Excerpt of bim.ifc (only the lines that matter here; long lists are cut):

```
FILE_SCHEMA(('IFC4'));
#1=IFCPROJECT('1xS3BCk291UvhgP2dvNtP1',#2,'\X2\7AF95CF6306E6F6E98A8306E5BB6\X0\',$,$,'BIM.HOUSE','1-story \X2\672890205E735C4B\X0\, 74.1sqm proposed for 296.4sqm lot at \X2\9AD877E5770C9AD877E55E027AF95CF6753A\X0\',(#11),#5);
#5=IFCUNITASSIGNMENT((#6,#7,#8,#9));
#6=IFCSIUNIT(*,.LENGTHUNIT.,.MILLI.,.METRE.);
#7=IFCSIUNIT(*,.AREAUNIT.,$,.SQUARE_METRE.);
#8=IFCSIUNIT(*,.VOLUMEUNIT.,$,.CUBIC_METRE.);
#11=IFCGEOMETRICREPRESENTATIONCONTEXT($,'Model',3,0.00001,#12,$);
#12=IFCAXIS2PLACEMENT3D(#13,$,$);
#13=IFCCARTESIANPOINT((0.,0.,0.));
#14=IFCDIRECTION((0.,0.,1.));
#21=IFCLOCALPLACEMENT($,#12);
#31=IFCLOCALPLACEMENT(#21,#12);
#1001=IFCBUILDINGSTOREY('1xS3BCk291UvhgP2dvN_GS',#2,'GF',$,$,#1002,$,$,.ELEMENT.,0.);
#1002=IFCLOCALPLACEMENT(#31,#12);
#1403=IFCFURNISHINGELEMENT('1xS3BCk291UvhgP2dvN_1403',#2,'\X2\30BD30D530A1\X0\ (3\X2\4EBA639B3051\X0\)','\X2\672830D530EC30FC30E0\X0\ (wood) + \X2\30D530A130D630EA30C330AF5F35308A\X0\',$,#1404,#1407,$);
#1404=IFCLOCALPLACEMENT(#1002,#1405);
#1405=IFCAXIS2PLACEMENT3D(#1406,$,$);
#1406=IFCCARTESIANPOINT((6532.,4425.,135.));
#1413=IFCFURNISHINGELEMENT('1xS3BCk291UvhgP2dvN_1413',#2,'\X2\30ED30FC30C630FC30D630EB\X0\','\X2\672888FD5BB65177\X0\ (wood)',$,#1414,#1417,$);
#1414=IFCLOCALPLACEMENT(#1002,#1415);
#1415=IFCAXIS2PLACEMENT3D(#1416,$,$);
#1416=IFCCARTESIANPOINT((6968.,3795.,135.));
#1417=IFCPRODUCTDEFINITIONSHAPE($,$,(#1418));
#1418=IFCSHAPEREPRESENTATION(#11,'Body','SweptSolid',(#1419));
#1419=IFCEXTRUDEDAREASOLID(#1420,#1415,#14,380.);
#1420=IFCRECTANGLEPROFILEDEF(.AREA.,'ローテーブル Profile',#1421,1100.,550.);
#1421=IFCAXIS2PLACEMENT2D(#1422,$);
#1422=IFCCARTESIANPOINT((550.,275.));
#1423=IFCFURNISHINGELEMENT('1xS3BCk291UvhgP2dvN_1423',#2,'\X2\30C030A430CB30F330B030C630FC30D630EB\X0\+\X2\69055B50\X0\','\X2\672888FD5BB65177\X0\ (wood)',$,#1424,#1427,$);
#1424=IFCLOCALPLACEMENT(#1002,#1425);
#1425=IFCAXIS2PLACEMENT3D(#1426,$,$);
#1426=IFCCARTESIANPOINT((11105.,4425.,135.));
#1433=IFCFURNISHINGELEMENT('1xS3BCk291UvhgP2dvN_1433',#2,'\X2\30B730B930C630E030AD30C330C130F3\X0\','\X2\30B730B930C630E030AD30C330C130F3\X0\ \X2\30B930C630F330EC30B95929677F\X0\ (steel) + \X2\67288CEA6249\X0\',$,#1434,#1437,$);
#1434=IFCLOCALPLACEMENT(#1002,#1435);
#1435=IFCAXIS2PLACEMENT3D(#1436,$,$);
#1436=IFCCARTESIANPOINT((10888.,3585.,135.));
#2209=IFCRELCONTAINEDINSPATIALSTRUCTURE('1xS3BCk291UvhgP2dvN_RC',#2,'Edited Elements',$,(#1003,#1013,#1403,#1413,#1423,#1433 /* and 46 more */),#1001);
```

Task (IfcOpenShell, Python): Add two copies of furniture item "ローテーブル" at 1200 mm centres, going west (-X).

```python
import numpy as np
import ifcopenshell
import ifcopenshell.api.geometry
import ifcopenshell.api.root
import ifcopenshell.util.element
import ifcopenshell.util.placement
import ifcopenshell.util.unit

model = ifcopenshell.open("bim.ifc")
unit_scale = ifcopenshell.util.unit.calculate_unit_scale(model)


def reuse_history(source, copy):
    """copy_class also copies each property set's owner history, people and application; keep the originals."""
    for rel in copy.IsDefinedBy:
        if rel.is_a("IfcRelDefinesByProperties") and (history := rel.RelatingPropertyDefinition.OwnerHistory):
            rel.RelatingPropertyDefinition.OwnerHistory = source.OwnerHistory
            ifcopenshell.util.element.remove_deep2(model, history)


source = model.by_guid("1xS3BCk291UvhgP2dvN_1413")
base = ifcopenshell.util.placement.get_local_placement(source.ObjectPlacement)
step = np.array([-1.0, 0.0, 0.0]) * 1.2 / unit_scale

for i in range(1, 3):
    copy = ifcopenshell.api.root.copy_class(model, product=source)
    copy.Representation = ifcopenshell.util.element.copy_deep(
        model, source.Representation, exclude=["IfcGeometricRepresentationContext", "IfcRepresentationMap"]
    )
    reuse_history(source, copy)
    matrix = base.copy()
    matrix[:3, 3] += i * step
    print("added at", matrix[:3, 3].round(3) + 0.0)
    ifcopenshell.api.geometry.edit_object_placement(model, product=copy, matrix=matrix, is_si=False)

model.write("bim-out.ifc")
```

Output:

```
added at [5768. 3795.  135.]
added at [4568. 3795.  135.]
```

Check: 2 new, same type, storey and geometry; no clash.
